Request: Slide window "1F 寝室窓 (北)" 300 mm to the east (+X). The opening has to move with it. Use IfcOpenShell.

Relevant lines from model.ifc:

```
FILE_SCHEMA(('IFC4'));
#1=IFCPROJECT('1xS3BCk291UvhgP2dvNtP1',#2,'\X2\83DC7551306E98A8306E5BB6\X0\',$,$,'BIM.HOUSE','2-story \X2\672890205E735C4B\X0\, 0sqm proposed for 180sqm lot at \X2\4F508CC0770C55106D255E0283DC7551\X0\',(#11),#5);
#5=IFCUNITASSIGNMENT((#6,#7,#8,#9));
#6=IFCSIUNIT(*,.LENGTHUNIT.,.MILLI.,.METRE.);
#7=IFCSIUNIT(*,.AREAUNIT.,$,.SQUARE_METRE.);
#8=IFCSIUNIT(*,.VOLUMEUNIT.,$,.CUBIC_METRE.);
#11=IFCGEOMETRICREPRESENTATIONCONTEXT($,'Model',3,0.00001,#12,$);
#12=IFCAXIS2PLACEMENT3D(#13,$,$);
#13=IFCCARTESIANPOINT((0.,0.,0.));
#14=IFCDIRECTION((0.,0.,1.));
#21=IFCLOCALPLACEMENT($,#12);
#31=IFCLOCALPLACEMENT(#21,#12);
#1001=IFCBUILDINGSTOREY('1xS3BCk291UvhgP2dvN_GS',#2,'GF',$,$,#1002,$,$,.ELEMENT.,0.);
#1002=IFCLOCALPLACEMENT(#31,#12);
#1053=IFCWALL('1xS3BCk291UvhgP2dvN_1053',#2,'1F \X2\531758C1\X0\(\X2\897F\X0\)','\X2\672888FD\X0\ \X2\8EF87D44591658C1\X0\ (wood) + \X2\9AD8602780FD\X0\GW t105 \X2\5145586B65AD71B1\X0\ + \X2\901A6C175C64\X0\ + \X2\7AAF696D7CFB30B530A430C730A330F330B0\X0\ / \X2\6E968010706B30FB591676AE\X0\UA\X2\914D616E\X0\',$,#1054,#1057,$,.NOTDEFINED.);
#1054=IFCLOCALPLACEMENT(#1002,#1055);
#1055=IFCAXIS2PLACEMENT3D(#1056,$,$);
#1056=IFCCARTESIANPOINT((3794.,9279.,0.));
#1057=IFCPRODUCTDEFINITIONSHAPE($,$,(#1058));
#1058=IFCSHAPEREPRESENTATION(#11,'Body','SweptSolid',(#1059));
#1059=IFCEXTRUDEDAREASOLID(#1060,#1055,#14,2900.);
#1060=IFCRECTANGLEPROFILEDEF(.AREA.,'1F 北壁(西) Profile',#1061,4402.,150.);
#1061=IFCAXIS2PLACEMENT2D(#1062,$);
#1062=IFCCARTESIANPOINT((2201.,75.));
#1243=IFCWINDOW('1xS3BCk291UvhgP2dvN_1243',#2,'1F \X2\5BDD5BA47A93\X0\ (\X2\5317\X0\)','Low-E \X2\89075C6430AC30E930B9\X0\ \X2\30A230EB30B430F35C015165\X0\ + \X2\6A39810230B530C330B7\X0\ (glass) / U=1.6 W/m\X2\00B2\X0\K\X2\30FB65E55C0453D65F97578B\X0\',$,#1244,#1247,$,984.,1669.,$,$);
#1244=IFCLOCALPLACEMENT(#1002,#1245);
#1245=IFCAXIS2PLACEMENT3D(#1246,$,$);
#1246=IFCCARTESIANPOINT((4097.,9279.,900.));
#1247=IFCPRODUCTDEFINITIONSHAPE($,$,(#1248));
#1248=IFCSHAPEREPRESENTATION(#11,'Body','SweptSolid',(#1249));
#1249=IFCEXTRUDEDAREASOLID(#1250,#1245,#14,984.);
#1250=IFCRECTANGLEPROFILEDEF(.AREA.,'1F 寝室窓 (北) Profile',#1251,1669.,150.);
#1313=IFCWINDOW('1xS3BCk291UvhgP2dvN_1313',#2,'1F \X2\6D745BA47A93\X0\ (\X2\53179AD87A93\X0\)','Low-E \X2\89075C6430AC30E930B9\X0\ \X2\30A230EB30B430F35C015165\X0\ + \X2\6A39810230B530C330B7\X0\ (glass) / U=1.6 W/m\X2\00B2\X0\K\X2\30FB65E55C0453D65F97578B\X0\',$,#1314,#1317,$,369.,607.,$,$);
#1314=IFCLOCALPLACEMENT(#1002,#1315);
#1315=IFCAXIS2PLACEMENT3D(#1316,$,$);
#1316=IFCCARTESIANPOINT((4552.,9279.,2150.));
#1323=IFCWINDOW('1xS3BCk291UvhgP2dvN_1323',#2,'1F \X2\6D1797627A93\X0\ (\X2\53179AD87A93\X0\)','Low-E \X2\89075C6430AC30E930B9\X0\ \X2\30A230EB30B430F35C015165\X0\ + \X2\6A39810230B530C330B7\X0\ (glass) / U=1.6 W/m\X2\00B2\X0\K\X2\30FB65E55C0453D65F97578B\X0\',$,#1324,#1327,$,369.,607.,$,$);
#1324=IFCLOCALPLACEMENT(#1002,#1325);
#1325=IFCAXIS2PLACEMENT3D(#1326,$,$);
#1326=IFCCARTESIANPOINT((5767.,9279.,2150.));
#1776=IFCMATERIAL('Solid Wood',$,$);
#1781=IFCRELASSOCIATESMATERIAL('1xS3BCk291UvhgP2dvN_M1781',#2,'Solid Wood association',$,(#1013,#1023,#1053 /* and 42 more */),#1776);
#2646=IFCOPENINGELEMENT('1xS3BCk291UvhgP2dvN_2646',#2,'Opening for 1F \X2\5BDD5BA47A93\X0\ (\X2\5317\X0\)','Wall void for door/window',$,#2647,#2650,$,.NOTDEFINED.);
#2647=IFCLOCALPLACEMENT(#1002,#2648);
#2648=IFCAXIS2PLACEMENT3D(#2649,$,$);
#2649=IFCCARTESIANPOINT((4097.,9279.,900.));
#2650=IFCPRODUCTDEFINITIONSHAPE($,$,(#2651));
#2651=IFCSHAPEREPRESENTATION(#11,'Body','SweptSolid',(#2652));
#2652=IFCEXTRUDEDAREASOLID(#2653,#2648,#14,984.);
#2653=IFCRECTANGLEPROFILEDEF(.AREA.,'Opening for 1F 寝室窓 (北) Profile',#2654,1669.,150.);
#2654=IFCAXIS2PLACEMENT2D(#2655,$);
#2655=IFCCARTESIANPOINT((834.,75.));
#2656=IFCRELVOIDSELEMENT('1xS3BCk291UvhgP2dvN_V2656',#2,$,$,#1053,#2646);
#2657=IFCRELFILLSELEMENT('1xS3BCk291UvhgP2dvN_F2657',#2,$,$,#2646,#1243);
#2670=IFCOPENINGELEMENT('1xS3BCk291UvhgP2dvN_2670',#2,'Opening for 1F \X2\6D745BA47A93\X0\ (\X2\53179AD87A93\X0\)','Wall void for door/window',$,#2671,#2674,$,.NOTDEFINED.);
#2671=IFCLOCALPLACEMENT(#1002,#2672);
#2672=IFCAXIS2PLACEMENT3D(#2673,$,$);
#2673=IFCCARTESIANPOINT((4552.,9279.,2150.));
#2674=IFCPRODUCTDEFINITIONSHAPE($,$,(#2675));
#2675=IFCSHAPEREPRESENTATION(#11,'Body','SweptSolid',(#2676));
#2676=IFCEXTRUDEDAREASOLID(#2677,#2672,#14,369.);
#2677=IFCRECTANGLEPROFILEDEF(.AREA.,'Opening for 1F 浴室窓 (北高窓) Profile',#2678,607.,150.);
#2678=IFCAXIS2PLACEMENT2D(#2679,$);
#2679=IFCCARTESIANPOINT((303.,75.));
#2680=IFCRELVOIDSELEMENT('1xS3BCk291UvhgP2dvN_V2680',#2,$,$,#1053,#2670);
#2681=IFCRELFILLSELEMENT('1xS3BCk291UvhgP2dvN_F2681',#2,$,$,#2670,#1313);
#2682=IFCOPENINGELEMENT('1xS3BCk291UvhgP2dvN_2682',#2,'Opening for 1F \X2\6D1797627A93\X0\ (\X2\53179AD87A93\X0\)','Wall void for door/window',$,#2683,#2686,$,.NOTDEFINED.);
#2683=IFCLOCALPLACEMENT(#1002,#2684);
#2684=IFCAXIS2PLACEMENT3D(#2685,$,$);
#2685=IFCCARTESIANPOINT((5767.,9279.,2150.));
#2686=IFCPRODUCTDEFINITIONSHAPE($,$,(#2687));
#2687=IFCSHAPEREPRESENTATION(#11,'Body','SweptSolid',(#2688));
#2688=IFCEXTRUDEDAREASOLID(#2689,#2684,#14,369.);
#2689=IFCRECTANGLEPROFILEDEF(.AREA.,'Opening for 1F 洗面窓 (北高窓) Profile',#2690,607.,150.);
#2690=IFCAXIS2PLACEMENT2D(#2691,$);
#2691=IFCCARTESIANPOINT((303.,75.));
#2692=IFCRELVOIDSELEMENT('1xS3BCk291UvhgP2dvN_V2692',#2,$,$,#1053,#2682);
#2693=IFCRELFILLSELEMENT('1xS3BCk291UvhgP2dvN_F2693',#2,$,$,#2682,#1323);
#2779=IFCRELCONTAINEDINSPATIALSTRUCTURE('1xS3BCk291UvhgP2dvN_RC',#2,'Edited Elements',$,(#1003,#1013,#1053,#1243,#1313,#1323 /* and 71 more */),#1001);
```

```python
import ifcopenshell
import ifcopenshell.api.geometry
import ifcopenshell.util.placement
import ifcopenshell.util.unit

model = ifcopenshell.open("model.ifc")
unit_scale = ifcopenshell.util.unit.calculate_unit_scale(model)

window = model.by_guid("1xS3BCk291UvhgP2dvN_1243")
opening = window.FillsVoids[0].RelatingOpeningElement
wall = opening.VoidsElements[0].RelatingBuildingElement

wall_matrix = ifcopenshell.util.placement.get_local_placement(wall.ObjectPlacement)
shift = wall_matrix[:3, 0] * 0.3 / unit_scale
before = ifcopenshell.util.placement.get_local_placement(window.ObjectPlacement)[:3, 3].copy()

# The window is not placed relative to its opening, so move both.
for product in (opening, window):
    matrix = ifcopenshell.util.placement.get_local_placement(product.ObjectPlacement)
    matrix[:3, 3] += shift
    ifcopenshell.api.geometry.edit_object_placement(model, product=product, matrix=matrix, is_si=False)

after = ifcopenshell.util.placement.get_local_placement(window.ObjectPlacement)[:3, 3]
print("window moved by", (after - before).round(3) + 0.0)

model.write("model_v2.ifc")
```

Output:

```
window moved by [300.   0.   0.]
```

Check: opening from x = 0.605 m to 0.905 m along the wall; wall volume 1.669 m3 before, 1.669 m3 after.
